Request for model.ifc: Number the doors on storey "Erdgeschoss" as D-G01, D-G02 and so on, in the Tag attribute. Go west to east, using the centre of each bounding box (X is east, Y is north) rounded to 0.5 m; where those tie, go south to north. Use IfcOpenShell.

First a look at what the model holds.

```python
import ifcopenshell
import ifcopenshell.util.element
import ifcopenshell.util.placement

model = ifcopenshell.open("model.ifc")
print(model.schema)
storey = next(s for s in model.by_type("IfcBuildingStorey") if s.Name == "Erdgeschoss")
doors = [e for e in ifcopenshell.util.element.get_decomposition(storey) if e.is_a("IfcDoor")]
for e in sorted(doors, key=lambda e: e.id()):
    origin = ifcopenshell.util.placement.get_local_placement(e.ObjectPlacement)[:3, 3]
    print(e.id(), e.Tag, e.Name, origin.round(2) + 0.0, sep=" | ")
```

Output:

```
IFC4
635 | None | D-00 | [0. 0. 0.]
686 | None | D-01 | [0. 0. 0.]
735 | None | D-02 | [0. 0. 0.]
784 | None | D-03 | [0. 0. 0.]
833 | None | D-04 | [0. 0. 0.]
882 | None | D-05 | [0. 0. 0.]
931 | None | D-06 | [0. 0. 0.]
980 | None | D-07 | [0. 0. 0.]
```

```python
import ifcopenshell
import ifcopenshell.geom
import ifcopenshell.util.element
import ifcopenshell.util.shape

model = ifcopenshell.open("model.ifc")
settings = ifcopenshell.geom.settings()
settings.set("use-world-coords", True)


def centre(element):
    shape = ifcopenshell.geom.create_shape(settings, element)
    return ifcopenshell.util.shape.get_bbox_centroid(shape.geometry)


storey = next(s for s in model.by_type("IfcBuildingStorey") if s.Name == "Erdgeschoss")
doors = [e for e in ifcopenshell.util.element.get_decomposition(storey) if e.is_a("IfcDoor")]

# Insertion points can sit at a corner or the storey origin, so sort by the geometry (in metres).
centres = {e: centre(e) for e in doors}
doors.sort(key=lambda e: (round(centres[e][0] / 0.5), centres[e][1]))

for i, e in enumerate(doors, start=1):
    number = f"D-G{i:02d}"
    e.Tag = number
    print(e.id(), number)

model.write("model_rev.ifc")
```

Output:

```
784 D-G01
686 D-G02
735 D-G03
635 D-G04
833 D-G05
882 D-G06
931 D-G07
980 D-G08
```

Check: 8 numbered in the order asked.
